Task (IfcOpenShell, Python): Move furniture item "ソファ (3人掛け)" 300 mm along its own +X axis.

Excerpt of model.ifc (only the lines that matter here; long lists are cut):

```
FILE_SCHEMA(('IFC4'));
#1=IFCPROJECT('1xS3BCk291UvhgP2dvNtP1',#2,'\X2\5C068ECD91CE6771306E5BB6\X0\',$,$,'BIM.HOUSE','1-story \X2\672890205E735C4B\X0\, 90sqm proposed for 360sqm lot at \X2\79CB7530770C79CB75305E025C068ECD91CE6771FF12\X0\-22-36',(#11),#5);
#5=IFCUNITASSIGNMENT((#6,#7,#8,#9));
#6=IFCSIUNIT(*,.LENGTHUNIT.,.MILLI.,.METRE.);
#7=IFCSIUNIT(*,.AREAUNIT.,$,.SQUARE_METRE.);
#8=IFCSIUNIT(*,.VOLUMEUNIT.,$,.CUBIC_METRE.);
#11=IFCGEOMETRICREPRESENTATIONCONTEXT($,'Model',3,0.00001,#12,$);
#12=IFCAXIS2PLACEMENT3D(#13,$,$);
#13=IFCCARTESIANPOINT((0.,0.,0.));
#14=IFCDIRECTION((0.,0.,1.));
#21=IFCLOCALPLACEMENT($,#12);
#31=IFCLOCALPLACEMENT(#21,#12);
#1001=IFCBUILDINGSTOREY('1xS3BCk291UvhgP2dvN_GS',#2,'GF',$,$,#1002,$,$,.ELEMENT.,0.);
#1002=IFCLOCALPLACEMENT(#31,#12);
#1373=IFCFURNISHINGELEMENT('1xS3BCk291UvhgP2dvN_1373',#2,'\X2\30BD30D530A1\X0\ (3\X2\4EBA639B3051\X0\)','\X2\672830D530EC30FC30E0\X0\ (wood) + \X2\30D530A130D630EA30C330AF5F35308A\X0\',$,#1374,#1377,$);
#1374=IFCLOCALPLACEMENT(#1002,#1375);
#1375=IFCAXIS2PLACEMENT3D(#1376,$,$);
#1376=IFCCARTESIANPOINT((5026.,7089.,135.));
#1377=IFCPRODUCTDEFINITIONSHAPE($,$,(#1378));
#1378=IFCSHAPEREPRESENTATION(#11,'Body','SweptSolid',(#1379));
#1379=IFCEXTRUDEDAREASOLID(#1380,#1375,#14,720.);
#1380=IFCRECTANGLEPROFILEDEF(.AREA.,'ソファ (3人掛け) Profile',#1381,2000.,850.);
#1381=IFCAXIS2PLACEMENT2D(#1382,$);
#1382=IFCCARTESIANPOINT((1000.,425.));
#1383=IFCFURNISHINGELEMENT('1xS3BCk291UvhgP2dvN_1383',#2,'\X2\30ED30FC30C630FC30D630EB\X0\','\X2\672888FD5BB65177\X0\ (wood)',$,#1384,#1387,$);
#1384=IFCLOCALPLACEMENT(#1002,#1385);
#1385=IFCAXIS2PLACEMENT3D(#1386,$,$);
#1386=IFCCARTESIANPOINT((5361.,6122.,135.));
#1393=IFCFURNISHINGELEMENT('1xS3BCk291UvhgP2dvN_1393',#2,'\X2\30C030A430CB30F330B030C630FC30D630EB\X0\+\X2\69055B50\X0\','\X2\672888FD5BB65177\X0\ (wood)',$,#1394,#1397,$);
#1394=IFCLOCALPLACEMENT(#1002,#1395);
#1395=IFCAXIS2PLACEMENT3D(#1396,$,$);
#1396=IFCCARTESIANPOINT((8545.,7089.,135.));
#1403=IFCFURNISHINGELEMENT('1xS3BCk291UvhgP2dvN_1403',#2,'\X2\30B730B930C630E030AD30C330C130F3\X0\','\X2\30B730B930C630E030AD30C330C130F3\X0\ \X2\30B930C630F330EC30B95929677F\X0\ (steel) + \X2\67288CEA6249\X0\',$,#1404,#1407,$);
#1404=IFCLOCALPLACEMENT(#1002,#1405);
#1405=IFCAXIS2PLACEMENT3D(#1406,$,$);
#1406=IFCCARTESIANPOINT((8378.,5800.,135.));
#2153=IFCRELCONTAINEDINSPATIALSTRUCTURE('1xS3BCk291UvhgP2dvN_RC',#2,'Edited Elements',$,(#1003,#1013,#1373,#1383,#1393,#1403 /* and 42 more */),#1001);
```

```python
import ifcopenshell
import ifcopenshell.api.geometry
import ifcopenshell.util.placement

model = ifcopenshell.open("model.ifc")

item = model.by_id(1373)
matrix = ifcopenshell.util.placement.get_local_placement(item.ObjectPlacement)
matrix[:3, 3] += matrix[:3, 0] * 300.0
ifcopenshell.api.geometry.edit_object_placement(model, product=item, matrix=matrix, is_si=False)

print(ifcopenshell.util.placement.get_local_placement(item.ObjectPlacement).round(3) + 0.0)

model.write("model_rev.ifc")
```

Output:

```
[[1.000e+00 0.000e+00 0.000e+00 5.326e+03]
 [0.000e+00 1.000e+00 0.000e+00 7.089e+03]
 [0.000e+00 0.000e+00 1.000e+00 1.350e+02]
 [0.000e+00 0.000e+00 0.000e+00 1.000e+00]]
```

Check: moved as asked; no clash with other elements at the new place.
